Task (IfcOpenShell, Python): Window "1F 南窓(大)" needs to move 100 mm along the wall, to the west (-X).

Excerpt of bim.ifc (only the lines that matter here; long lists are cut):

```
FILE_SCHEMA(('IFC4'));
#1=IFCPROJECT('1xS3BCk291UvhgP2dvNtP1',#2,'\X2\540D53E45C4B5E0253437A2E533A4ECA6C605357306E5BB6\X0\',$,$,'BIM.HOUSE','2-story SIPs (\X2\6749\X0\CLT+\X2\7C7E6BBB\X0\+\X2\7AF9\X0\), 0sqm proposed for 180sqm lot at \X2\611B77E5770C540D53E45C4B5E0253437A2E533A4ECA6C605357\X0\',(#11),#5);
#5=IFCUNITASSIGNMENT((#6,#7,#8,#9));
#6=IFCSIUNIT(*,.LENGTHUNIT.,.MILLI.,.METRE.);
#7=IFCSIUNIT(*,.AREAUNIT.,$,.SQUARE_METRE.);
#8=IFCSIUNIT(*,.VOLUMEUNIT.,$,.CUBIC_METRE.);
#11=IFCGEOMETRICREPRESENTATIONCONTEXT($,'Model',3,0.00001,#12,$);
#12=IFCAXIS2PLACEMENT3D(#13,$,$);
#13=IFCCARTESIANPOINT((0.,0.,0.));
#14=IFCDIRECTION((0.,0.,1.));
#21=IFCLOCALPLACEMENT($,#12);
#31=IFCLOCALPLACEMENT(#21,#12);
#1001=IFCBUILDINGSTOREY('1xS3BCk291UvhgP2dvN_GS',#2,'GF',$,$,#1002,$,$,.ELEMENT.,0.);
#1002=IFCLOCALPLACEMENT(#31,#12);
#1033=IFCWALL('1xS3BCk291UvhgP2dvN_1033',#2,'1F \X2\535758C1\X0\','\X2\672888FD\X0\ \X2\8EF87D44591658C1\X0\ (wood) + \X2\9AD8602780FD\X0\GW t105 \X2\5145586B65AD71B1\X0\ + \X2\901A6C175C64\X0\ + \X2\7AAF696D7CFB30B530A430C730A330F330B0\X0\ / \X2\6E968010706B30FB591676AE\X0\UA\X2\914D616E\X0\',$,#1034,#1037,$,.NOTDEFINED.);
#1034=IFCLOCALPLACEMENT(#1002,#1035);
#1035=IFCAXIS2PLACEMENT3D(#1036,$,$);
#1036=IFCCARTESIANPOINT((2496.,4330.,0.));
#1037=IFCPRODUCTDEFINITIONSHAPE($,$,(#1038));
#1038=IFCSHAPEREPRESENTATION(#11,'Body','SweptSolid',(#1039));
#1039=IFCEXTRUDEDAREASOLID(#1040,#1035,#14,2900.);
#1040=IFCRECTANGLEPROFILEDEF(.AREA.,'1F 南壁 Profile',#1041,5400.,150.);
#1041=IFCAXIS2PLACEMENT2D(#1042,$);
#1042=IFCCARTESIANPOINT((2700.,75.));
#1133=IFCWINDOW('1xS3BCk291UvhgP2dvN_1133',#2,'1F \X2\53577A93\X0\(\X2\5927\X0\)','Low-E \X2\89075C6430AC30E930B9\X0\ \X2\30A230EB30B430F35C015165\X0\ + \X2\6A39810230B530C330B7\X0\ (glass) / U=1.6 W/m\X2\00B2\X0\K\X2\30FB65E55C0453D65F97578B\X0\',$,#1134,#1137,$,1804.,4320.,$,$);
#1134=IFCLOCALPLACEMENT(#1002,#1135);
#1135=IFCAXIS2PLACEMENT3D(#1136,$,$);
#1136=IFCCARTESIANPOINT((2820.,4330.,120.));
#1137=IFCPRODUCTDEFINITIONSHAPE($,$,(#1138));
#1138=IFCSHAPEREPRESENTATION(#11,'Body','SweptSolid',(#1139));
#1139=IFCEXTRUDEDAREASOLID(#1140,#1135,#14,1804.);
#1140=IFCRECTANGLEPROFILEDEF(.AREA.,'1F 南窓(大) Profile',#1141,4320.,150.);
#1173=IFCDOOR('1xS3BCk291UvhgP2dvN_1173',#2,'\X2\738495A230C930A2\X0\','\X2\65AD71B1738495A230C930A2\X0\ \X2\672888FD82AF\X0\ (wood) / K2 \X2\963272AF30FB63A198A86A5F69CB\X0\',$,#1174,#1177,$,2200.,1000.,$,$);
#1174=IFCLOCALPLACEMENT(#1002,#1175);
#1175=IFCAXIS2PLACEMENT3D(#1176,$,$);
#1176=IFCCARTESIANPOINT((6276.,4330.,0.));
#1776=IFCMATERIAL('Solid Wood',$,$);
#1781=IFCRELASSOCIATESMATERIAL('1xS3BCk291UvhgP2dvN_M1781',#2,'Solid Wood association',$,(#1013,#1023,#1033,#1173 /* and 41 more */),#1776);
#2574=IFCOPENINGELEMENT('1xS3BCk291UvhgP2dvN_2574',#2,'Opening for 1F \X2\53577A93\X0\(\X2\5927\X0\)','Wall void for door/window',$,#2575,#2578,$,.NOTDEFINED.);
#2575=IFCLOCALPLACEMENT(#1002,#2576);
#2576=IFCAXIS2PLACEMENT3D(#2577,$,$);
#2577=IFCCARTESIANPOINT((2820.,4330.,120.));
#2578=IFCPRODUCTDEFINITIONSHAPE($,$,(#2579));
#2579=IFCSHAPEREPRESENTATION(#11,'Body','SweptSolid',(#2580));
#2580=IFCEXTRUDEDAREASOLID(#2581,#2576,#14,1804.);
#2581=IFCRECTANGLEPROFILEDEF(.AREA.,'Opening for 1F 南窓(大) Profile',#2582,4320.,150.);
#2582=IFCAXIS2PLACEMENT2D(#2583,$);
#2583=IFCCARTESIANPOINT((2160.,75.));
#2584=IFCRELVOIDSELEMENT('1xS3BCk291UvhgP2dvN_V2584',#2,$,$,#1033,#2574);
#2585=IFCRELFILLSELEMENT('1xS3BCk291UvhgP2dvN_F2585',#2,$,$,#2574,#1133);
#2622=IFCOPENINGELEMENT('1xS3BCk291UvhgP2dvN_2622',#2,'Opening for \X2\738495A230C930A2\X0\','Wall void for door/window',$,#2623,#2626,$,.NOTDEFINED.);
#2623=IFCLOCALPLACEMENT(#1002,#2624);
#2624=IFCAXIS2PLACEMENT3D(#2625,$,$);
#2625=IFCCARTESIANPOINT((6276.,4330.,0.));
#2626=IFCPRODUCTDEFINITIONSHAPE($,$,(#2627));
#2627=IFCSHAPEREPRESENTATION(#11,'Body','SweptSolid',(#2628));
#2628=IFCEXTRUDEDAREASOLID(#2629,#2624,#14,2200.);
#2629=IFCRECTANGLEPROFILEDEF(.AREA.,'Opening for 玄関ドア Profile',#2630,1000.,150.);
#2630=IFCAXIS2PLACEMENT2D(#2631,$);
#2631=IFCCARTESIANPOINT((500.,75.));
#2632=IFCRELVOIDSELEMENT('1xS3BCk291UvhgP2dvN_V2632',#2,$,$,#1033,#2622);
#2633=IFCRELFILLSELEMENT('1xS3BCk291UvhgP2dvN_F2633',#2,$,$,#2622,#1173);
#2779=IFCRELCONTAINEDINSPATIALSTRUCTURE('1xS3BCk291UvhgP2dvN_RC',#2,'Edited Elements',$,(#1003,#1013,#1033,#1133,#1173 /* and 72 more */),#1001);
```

```python
import ifcopenshell
import ifcopenshell.api.geometry
import ifcopenshell.util.placement
import ifcopenshell.util.unit

model = ifcopenshell.open("bim.ifc")
unit_scale = ifcopenshell.util.unit.calculate_unit_scale(model)

window = model.by_guid("1xS3BCk291UvhgP2dvN_1133")
opening = window.FillsVoids[0].RelatingOpeningElement
wall = opening.VoidsElements[0].RelatingBuildingElement

wall_matrix = ifcopenshell.util.placement.get_local_placement(wall.ObjectPlacement)
shift = wall_matrix[:3, 0] * -0.1 / unit_scale
before = ifcopenshell.util.placement.get_local_placement(window.ObjectPlacement)[:3, 3].copy()

# The window is not placed relative to its opening, so move both.
for product in (opening, window):
    matrix = ifcopenshell.util.placement.get_local_placement(product.ObjectPlacement)
    matrix[:3, 3] += shift
    ifcopenshell.api.geometry.edit_object_placement(model, product=product, matrix=matrix, is_si=False)

after = ifcopenshell.util.placement.get_local_placement(window.ObjectPlacement)[:3, 3]
print("window moved by", (after - before).round(3) + 0.0)

model.write("bim_edited.ifc")
```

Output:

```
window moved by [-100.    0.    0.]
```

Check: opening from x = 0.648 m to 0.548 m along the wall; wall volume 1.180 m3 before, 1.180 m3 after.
